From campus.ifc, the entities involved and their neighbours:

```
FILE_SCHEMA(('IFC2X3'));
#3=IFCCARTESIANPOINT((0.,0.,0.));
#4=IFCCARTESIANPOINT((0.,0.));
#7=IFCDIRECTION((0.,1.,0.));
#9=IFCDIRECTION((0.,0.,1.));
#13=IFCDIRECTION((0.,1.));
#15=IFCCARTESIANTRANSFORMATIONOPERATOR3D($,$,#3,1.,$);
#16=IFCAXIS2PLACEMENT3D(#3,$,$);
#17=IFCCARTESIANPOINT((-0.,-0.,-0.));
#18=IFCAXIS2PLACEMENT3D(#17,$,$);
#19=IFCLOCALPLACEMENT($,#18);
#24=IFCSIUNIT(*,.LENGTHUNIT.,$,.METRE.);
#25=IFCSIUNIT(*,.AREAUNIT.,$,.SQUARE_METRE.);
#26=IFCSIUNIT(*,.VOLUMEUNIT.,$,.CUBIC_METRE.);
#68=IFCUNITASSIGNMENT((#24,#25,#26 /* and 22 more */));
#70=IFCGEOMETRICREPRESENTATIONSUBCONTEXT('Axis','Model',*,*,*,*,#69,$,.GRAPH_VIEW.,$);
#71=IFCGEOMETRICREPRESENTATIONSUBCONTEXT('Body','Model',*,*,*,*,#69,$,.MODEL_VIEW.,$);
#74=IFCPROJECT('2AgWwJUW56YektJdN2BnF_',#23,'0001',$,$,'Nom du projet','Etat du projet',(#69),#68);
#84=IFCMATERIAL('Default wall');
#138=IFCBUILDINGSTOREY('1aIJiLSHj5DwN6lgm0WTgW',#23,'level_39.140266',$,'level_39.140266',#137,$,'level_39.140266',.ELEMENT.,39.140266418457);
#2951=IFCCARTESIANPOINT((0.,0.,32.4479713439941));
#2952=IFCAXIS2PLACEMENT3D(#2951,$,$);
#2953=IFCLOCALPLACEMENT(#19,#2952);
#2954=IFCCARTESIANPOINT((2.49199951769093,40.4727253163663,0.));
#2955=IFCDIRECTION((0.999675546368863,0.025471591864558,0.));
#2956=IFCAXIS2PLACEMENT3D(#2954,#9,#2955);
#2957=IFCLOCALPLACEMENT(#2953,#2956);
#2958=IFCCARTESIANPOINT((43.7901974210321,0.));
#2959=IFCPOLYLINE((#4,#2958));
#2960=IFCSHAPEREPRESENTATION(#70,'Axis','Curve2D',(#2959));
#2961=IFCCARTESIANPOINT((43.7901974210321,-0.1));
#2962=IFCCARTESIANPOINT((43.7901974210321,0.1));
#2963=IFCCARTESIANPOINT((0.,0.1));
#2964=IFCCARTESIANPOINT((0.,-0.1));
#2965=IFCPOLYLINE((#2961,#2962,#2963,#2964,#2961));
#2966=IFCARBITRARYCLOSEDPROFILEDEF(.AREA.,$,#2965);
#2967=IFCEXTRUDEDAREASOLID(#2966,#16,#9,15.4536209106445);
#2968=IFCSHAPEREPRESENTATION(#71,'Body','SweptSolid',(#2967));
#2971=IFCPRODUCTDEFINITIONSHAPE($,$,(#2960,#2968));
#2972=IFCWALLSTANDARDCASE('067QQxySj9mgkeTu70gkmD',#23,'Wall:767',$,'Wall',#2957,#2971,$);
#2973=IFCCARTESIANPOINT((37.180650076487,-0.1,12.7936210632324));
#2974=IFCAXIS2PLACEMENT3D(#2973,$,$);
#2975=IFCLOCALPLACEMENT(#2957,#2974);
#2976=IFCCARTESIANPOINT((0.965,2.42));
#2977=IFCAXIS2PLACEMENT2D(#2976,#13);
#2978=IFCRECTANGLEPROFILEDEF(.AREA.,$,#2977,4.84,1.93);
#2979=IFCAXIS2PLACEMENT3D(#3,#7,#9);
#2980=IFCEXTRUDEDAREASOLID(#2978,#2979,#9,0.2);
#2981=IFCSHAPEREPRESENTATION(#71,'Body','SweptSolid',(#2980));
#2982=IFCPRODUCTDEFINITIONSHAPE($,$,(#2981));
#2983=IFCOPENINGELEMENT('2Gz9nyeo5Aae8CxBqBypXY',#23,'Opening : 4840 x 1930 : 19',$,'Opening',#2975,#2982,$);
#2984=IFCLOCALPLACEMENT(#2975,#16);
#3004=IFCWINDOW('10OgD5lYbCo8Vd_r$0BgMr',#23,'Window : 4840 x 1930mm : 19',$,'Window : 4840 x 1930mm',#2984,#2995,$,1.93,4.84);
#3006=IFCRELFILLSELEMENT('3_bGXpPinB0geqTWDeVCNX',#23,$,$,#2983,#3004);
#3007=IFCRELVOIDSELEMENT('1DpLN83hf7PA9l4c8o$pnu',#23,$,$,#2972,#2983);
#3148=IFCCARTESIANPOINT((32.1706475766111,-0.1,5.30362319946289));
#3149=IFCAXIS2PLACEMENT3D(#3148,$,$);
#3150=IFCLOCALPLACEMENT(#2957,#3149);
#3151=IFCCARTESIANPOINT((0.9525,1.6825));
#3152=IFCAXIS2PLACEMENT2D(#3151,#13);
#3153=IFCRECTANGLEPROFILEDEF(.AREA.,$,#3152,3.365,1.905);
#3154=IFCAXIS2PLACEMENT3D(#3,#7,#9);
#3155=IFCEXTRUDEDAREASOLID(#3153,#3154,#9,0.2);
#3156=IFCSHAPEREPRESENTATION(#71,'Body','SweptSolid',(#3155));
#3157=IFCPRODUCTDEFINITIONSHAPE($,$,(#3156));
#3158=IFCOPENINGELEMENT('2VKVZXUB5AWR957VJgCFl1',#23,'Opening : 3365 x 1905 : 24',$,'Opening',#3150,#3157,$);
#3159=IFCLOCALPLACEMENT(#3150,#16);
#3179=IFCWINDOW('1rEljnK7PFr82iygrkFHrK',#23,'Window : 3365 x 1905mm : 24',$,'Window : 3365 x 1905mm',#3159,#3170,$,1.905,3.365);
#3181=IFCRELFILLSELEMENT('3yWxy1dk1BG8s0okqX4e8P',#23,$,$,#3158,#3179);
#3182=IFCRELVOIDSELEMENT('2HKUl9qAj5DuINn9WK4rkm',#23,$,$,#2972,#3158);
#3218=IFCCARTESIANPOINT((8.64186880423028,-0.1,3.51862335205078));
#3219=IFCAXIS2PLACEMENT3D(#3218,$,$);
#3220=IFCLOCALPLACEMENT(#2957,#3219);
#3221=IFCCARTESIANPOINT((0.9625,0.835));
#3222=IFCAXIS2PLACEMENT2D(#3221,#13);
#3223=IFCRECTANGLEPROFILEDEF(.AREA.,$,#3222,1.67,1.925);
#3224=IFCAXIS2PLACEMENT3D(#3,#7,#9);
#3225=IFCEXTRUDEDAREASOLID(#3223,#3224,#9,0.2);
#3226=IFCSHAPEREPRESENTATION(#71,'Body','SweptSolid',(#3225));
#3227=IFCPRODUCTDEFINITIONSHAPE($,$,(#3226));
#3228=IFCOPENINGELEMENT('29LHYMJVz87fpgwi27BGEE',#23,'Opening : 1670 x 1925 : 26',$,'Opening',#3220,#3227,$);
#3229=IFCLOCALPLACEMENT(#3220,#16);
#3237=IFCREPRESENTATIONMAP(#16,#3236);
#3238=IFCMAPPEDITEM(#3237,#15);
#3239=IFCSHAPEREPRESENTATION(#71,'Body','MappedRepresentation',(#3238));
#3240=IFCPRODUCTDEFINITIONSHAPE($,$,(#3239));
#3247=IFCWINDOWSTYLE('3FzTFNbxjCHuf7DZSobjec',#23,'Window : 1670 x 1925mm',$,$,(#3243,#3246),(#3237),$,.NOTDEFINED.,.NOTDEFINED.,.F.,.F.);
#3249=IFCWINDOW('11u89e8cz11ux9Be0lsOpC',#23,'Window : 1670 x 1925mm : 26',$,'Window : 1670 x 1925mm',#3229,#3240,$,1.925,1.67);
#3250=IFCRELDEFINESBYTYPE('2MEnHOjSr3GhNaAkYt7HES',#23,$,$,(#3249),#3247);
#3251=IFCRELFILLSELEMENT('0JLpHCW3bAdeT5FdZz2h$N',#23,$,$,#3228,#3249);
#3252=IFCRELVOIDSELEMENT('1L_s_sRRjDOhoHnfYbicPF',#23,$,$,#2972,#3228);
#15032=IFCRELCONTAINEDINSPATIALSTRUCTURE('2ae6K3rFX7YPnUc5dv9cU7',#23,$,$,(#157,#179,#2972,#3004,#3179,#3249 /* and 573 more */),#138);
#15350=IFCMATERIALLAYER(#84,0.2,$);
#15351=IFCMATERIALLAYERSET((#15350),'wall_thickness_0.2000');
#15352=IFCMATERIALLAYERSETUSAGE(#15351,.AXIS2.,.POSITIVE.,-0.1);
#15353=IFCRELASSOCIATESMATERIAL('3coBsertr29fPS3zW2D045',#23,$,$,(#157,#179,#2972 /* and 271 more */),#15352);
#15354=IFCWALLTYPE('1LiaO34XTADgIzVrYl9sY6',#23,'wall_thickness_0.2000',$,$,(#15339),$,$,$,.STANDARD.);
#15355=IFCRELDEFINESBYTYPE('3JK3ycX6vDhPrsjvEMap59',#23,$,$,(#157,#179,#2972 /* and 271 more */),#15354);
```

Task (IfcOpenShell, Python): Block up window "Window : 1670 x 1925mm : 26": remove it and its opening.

```python
import ifcopenshell
import ifcopenshell.api.feature
import ifcopenshell.api.root
import ifcopenshell.geom
import ifcopenshell.util.shape

model = ifcopenshell.open("campus.ifc")
settings = ifcopenshell.geom.settings()


def volume(element):
    """Net volume in cubic metres, openings subtracted."""
    shape = ifcopenshell.geom.create_shape(settings, element)
    return ifcopenshell.util.shape.get_volume(shape.geometry)


window = model.by_guid("11u89e8cz11ux9Be0lsOpC")
opening = window.FillsVoids[0].RelatingOpeningElement
wall = opening.VoidsElements[0].RelatingBuildingElement
before = volume(wall)

ifcopenshell.api.root.remove_product(model, product=window)
ifcopenshell.api.feature.remove_feature(model, feature=opening)

after = volume(wall)

print(f"wall volume {before:.3f} -> {after:.3f} m3")

model.write("campus_updated.ifc")
```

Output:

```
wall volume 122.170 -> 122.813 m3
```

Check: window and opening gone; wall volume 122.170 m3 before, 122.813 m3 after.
